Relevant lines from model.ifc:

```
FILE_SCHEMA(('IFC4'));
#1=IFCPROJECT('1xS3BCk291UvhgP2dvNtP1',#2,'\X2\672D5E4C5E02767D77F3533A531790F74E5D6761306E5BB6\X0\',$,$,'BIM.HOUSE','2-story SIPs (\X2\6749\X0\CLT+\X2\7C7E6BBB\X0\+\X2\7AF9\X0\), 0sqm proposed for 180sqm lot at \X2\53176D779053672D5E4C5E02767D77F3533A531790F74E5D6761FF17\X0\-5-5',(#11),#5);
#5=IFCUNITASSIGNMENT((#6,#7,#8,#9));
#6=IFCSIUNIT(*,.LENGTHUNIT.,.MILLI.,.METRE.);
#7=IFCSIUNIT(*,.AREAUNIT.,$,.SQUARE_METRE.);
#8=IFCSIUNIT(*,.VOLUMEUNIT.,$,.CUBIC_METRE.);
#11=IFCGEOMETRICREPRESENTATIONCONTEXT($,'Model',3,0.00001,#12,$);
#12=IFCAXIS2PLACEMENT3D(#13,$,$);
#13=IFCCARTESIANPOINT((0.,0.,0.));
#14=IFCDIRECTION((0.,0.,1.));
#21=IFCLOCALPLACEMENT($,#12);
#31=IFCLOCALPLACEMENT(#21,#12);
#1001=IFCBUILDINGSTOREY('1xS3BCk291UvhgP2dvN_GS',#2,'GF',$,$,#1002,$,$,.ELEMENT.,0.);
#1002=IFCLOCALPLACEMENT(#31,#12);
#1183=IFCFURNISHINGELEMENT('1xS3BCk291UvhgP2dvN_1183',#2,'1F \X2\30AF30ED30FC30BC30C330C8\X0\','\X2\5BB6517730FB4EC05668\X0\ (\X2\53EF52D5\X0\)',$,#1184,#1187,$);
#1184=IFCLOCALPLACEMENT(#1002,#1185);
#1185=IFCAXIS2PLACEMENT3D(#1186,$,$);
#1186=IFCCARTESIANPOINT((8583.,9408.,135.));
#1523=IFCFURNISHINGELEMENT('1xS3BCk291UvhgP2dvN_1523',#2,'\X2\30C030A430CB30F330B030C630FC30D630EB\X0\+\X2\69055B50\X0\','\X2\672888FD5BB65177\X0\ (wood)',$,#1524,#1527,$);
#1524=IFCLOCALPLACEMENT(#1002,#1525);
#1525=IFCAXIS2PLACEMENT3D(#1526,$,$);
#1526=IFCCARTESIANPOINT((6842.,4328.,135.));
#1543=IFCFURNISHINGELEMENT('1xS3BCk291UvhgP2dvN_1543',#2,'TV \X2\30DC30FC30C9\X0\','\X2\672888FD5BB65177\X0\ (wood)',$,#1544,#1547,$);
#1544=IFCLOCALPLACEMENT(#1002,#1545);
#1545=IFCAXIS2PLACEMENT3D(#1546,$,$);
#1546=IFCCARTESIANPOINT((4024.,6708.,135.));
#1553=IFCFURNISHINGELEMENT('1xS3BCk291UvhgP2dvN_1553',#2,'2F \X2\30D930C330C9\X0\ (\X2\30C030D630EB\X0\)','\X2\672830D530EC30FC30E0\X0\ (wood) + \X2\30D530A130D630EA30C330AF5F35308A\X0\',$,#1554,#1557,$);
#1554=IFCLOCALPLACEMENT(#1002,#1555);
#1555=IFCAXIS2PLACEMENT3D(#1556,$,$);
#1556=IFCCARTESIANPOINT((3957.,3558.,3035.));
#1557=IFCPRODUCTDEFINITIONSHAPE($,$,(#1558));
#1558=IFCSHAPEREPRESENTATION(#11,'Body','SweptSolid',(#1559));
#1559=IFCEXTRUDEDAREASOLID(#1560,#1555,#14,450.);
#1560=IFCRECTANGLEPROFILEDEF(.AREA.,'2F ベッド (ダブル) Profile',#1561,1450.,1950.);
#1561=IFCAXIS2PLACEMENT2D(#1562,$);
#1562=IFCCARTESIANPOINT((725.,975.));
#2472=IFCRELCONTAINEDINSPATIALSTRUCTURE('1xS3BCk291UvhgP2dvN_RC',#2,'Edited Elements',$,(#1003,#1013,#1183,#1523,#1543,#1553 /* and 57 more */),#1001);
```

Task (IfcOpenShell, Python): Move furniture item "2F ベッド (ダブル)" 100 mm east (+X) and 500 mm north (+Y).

```python
import ifcopenshell
import ifcopenshell.api.geometry
import ifcopenshell.util.placement

model = ifcopenshell.open("model.ifc")

item = model.by_guid("1xS3BCk291UvhgP2dvN_1553")
matrix = ifcopenshell.util.placement.get_local_placement(item.ObjectPlacement)
matrix[0, 3] += 100.0
matrix[1, 3] += 500.0
ifcopenshell.api.geometry.edit_object_placement(model, product=item, matrix=matrix, is_si=False)

print(ifcopenshell.util.placement.get_local_placement(item.ObjectPlacement).round(3) + 0.0)

model.write("model_v2.ifc")
```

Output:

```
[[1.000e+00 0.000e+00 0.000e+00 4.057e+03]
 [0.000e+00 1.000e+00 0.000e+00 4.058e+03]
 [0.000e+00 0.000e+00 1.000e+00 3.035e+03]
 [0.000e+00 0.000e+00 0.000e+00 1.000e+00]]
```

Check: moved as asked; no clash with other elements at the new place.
